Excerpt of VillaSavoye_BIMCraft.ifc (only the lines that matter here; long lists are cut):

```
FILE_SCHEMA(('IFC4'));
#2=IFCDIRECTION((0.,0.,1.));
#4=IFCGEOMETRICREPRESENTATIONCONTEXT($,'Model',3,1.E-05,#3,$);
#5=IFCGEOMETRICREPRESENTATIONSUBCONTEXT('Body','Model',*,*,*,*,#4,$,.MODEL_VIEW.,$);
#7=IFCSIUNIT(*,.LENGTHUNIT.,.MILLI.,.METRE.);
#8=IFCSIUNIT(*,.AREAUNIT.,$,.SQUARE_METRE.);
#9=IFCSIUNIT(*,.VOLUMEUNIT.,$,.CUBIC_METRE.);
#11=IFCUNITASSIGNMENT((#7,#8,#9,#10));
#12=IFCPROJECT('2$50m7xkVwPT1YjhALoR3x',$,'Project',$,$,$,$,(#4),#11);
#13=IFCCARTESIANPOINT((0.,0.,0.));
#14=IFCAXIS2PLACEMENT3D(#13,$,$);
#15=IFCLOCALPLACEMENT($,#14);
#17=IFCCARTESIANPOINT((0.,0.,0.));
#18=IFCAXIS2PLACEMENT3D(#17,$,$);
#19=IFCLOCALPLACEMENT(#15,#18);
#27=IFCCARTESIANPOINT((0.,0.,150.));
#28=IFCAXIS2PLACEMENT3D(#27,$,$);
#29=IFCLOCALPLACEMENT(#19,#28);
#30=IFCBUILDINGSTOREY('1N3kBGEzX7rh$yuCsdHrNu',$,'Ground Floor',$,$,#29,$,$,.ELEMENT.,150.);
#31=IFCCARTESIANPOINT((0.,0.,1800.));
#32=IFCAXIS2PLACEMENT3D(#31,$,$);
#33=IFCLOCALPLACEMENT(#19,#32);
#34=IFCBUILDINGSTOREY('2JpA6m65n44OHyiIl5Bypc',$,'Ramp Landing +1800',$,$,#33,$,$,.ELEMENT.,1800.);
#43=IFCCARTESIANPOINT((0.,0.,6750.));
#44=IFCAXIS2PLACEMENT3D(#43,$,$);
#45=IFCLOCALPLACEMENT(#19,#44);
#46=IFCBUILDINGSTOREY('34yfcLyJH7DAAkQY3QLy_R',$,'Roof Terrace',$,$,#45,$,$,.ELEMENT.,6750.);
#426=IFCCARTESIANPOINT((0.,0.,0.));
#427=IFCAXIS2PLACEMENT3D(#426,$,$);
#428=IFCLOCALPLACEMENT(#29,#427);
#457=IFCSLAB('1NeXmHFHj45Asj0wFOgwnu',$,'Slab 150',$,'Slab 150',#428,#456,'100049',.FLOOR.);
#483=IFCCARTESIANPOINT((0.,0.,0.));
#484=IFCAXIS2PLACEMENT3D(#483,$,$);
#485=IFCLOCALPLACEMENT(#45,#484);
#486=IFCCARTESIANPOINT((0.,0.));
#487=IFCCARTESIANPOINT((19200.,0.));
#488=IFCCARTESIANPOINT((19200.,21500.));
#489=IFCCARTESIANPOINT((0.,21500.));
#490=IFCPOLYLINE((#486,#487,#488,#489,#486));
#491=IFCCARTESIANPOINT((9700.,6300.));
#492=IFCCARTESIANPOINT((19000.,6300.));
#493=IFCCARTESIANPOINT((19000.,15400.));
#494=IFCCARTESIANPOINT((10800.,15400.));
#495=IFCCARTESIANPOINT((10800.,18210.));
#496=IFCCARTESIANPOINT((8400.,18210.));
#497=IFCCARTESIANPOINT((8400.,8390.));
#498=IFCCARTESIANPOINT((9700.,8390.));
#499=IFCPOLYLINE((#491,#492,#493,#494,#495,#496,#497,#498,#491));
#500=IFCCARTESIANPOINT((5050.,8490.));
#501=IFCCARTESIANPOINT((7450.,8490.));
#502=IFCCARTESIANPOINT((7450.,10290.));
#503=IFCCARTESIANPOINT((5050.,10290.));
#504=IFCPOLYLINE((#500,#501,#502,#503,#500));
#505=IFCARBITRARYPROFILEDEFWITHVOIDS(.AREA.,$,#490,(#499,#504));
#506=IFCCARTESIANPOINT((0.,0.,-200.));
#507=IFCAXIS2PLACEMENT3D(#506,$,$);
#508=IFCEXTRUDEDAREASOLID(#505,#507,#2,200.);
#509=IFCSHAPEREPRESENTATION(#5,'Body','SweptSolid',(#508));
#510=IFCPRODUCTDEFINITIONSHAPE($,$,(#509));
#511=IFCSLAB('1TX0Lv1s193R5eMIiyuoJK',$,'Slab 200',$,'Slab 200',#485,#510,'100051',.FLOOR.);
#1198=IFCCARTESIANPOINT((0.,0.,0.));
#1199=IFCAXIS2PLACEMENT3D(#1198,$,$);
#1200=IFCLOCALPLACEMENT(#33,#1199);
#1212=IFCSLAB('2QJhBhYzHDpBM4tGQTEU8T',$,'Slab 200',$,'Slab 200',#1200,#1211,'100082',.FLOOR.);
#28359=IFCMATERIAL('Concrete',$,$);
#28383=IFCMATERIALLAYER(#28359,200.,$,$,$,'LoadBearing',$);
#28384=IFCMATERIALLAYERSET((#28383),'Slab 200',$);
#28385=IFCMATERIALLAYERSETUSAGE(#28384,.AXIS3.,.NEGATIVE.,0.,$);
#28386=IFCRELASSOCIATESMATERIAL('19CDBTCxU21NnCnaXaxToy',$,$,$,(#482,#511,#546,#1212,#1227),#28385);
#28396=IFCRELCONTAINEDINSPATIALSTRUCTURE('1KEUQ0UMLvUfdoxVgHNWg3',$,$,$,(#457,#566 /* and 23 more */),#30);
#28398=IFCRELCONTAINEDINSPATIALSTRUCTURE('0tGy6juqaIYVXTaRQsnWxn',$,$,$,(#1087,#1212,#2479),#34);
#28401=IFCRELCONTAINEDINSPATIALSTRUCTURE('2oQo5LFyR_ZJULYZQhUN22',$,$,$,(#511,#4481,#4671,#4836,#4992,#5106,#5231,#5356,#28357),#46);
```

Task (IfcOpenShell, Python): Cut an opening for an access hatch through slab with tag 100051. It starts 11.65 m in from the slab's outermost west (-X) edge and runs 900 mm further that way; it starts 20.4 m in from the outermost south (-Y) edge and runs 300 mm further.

```python
import numpy as np
import ifcopenshell
import ifcopenshell.api.feature
import ifcopenshell.api.geometry
import ifcopenshell.api.root
import ifcopenshell.geom
import ifcopenshell.util.placement
import ifcopenshell.util.representation
import ifcopenshell.util.shape
import ifcopenshell.util.unit

model = ifcopenshell.open("VillaSavoye_BIMCraft.ifc")
unit_scale = ifcopenshell.util.unit.calculate_unit_scale(model)
settings = ifcopenshell.geom.settings()


def volume(element):
    """Net volume in cubic metres, openings subtracted."""
    shape = ifcopenshell.geom.create_shape(settings, element)
    return ifcopenshell.util.shape.get_volume(shape.geometry)


slab = model.by_guid("1TX0Lv1s193R5eMIiyuoJK")
before = volume(slab)

# Extent in the slab's own axes, in metres. The edges named are its -X and -Y sides.
slab_shape = ifcopenshell.geom.create_shape(settings, slab)
vertices = ifcopenshell.util.shape.get_vertices(slab_shape.geometry)
x_min, y_min, bottom = vertices.min(axis=0)
top = vertices[:, 2].max()

opening = ifcopenshell.api.root.create_entity(model, ifc_class="IfcOpeningElement", name="Access hatch opening", predefined_type="OPENING")
context = ifcopenshell.util.representation.get_context(model, "Model", "Body", "MODEL_VIEW")
width, depth = 0.9, 0.3
outline = [(0.0, 0.0), (width, 0.0), (width, depth), (0.0, depth), (0.0, 0.0)]
# Overshoot both faces by 50 mm so the cut is clean.
shape = ifcopenshell.api.geometry.add_slab_representation(
    model, context=context, depth=top - bottom + 0.1, polyline=outline
)
ifcopenshell.api.geometry.assign_representation(model, product=opening, representation=shape)

matrix = ifcopenshell.util.placement.get_local_placement(slab.ObjectPlacement)
matrix[:, 3] = matrix @ np.append(np.array([x_min + 11.65, y_min + 20.4, bottom - 0.05]) / unit_scale, 1.0)
ifcopenshell.api.geometry.edit_object_placement(model, product=opening, matrix=matrix, is_si=False)
ifcopenshell.api.feature.add_feature(model, feature=opening, element=slab)

after = volume(slab)

print(f"slab volume {before:.3f} -> {after:.3f} m3")

model.write("VillaSavoye_BIMCraft-out.ifc")
```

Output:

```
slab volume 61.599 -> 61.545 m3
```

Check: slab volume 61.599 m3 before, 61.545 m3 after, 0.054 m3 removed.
